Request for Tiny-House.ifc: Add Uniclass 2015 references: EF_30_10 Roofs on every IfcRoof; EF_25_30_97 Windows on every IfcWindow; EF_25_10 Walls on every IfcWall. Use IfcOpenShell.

First a look at what the model holds.

```python
import ifcopenshell

model = ifcopenshell.open("Tiny-House.ifc")
print(model.schema)
print("classifications:", [c.Name for c in model.by_type("IfcClassification")])
for ifc_class in ("IfcDoor", "IfcRoof", "IfcStair", "IfcWall", "IfcWindow"):
    print(ifc_class, len(model.by_type(ifc_class)))
```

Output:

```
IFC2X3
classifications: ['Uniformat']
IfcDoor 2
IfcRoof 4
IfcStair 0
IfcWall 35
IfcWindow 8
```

```python
import ifcopenshell
import ifcopenshell.api.classification

model = ifcopenshell.open("Tiny-House.ifc")

# IFC2X3 requires Source and Edition and has no link from the project to the system.
system = model.create_entity("IfcClassification", Source="NBS", Edition="2015", Name="Uniclass 2015")

codes = {
    "IfcRoof": ("EF_30_10", "Roofs"),
    "IfcWindow": ("EF_25_30_97", "Windows"),
    "IfcWall": ("EF_25_10", "Walls"),
}
for ifc_class, (code, name) in codes.items():
    products = model.by_type(ifc_class)
    ifcopenshell.api.classification.add_reference(
        model, products=products, classification=system, identification=code, name=name
    )
    print(code, len(products))

model.write("Tiny-House_updated.ifc")
```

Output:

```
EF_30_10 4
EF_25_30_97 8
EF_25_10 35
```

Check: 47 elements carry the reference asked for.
